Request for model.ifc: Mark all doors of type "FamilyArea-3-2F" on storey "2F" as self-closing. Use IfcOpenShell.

First a look at what the model holds.

```python
import ifcopenshell
import ifcopenshell.util.element

model = ifcopenshell.open("model.ifc")
print(model.schema)
storey = next(s for s in model.by_type("IfcBuildingStorey") if s.Name == "2F")
doors = [e for e in ifcopenshell.util.element.get_decomposition(storey) if e.is_a("IfcDoor")]
seen = {}
for e in doors:
    element_type = ifcopenshell.util.element.get_type(e)
    key = (element_type.Name if element_type != e and element_type else None, ifcopenshell.util.element.get_pset(e, "Pset_DoorCommon", "SelfClosing"))
    seen[key] = seen.get(key, 0) + 1
for (name, value), count in sorted(seen.items(), key=str):
    print(count, "x", name, "|", value)
```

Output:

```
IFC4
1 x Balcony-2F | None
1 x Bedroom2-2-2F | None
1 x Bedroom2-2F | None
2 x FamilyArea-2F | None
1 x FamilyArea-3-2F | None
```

```python
import ifcopenshell
import ifcopenshell.api.pset
import ifcopenshell.util.element

model = ifcopenshell.open("model.ifc")

storey = next(s for s in model.by_type("IfcBuildingStorey") if s.Name == "2F")
doors = [e for e in ifcopenshell.util.element.get_decomposition(storey) if e.is_a("IfcDoor")]

count = 0
for e in doors:
    element_type = ifcopenshell.util.element.get_type(e)
    if element_type in (None, e) or element_type.Name != "FamilyArea-3-2F":
        continue
    # add_pset returns the element's existing set when there is one.
    pset = ifcopenshell.api.pset.add_pset(model, product=e, name="Pset_DoorCommon")
    ifcopenshell.api.pset.edit_pset(model, pset=pset, properties={"SelfClosing": True})
    count += 1

print(count, "doors updated")

model.write("model_updated.ifc")
```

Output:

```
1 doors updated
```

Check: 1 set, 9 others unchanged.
